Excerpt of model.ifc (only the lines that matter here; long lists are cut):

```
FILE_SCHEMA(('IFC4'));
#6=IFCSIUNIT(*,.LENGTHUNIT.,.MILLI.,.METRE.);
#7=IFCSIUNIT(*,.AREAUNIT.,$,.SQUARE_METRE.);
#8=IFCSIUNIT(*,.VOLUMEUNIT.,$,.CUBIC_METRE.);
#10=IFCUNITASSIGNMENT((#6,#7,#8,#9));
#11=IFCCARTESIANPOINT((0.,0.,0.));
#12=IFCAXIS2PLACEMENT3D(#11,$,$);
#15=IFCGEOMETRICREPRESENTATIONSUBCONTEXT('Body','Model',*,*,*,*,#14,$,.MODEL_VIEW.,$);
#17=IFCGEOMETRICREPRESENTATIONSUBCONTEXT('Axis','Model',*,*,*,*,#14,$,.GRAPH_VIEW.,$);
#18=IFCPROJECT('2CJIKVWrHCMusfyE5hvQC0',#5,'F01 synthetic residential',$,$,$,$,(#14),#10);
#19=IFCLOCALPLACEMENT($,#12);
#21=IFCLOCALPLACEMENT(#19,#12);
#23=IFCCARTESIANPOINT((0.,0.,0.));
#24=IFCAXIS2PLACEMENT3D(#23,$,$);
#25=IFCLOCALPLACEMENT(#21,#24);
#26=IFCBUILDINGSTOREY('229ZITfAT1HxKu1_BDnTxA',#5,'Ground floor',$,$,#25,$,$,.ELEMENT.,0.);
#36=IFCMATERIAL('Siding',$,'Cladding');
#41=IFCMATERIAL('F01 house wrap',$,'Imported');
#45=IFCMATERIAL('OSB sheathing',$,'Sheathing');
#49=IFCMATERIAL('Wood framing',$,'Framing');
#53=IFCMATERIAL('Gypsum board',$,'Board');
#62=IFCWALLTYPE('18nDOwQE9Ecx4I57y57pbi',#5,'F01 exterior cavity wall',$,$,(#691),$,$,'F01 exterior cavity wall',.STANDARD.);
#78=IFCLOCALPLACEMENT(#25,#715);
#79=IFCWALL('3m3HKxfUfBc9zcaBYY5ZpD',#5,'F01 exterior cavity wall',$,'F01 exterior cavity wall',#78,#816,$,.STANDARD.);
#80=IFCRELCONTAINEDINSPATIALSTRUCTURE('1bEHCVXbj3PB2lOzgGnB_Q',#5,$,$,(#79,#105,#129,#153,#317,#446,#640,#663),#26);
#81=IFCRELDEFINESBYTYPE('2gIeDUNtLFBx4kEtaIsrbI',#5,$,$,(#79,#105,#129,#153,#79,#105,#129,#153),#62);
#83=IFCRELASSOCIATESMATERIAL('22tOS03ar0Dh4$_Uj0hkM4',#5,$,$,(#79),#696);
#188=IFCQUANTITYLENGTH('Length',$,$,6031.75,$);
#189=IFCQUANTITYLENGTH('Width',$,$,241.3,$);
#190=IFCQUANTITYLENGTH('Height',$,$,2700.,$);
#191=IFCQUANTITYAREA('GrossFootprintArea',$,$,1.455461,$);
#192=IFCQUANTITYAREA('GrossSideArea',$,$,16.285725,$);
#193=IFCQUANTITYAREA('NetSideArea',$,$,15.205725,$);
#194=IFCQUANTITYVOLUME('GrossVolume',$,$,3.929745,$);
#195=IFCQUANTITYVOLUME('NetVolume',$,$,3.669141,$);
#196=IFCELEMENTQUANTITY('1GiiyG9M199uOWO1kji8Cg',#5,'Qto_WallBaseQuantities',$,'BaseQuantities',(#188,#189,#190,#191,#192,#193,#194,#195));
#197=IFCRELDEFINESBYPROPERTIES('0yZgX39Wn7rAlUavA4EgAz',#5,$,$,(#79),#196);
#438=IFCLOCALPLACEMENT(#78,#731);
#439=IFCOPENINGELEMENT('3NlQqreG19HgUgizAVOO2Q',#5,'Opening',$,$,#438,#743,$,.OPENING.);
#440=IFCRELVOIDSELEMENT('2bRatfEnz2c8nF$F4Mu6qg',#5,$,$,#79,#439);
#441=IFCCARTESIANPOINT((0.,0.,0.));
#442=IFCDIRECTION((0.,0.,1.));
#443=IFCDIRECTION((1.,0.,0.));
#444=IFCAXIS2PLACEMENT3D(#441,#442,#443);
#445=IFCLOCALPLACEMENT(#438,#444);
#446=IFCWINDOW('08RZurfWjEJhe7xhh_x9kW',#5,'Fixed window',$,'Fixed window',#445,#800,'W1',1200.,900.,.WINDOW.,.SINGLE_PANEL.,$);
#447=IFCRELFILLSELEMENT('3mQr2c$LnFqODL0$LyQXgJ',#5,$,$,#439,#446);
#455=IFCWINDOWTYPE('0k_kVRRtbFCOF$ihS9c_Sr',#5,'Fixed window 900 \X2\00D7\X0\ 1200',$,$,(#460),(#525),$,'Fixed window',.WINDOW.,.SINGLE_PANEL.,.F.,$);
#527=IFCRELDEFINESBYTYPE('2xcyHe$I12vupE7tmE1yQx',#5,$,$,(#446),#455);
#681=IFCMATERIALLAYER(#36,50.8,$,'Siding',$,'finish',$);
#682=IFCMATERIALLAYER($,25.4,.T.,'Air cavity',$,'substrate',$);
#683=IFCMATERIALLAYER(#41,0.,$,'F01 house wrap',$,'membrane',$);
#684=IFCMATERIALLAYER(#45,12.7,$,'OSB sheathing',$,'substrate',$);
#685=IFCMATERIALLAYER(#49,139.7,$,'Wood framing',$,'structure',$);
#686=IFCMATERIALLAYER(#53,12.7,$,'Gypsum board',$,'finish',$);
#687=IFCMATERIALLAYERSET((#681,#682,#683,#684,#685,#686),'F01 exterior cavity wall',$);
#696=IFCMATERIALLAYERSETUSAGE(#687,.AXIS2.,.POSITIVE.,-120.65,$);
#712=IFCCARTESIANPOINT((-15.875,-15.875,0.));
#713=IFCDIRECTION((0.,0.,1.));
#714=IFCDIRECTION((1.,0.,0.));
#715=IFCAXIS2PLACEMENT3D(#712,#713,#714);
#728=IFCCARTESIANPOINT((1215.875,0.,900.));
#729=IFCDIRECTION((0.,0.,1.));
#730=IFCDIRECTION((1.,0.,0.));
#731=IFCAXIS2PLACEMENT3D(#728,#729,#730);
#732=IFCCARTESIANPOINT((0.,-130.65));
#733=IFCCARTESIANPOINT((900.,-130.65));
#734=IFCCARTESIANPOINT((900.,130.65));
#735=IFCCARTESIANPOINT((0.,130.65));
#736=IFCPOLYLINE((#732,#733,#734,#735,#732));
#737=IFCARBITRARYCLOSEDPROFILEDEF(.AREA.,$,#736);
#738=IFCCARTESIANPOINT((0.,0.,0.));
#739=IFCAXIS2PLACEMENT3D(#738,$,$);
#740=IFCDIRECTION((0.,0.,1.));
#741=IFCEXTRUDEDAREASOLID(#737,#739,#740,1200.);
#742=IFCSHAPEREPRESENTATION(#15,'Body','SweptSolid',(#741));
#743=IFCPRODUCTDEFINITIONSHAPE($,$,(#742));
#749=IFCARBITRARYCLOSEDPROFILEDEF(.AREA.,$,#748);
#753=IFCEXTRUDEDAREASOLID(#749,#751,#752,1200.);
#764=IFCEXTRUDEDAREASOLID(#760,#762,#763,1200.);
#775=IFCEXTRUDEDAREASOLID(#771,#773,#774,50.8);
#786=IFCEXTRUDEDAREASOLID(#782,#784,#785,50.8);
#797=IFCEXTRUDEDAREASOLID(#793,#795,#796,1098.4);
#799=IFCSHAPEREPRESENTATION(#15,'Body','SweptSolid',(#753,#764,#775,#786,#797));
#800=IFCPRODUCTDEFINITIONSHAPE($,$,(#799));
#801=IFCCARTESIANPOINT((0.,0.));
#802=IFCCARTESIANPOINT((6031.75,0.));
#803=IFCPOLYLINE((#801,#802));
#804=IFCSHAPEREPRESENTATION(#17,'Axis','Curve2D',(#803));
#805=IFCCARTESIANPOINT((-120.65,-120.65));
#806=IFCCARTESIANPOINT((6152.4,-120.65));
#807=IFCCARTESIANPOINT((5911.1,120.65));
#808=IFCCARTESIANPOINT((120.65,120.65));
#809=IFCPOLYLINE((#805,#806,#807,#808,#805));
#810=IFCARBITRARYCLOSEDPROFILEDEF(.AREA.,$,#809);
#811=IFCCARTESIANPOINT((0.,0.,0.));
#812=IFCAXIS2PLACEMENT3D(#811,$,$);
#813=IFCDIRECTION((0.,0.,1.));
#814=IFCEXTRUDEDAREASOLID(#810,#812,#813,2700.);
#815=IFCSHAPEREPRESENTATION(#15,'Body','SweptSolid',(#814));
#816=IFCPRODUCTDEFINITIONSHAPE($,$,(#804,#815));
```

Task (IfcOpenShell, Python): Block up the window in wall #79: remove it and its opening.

```python
import ifcopenshell
import ifcopenshell.api.feature
import ifcopenshell.api.pset
import ifcopenshell.api.root
import ifcopenshell.geom
import ifcopenshell.util.element
import ifcopenshell.util.shape
import ifcopenshell.util.unit

model = ifcopenshell.open("model.ifc")
area_scale = ifcopenshell.util.unit.calculate_unit_scale(model, "AREAUNIT")
volume_scale = ifcopenshell.util.unit.calculate_unit_scale(model, "VOLUMEUNIT")
settings = ifcopenshell.geom.settings()


def volume(element):
    """Net volume in cubic metres, openings subtracted."""
    shape = ifcopenshell.geom.create_shape(settings, element)
    return ifcopenshell.util.shape.get_volume(shape.geometry)


window = model.by_id(446)
opening = window.FillsVoids[0].RelatingOpeningElement
wall = opening.VoidsElements[0].RelatingBuildingElement
before = volume(wall)

ifcopenshell.api.root.remove_product(model, product=window)
ifcopenshell.api.feature.remove_feature(model, feature=opening)

after = volume(wall)
thickness = 0.2413  # wall thickness in metres

# Update the wall's stored quantities.
qto = model.by_id(ifcopenshell.util.element.get_pset(wall, "Qto_WallBaseQuantities", should_inherit=False)["id"])
ifcopenshell.api.pset.edit_qto(model, qto=qto, properties={
    "NetSideArea": after / thickness / area_scale,
    "NetVolume": after / volume_scale,
})

print(f"wall volume {before:.3f} -> {after:.3f} m3")

model.write("model_updated.ifc")
```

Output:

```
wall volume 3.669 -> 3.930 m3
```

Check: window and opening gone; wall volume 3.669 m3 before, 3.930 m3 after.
